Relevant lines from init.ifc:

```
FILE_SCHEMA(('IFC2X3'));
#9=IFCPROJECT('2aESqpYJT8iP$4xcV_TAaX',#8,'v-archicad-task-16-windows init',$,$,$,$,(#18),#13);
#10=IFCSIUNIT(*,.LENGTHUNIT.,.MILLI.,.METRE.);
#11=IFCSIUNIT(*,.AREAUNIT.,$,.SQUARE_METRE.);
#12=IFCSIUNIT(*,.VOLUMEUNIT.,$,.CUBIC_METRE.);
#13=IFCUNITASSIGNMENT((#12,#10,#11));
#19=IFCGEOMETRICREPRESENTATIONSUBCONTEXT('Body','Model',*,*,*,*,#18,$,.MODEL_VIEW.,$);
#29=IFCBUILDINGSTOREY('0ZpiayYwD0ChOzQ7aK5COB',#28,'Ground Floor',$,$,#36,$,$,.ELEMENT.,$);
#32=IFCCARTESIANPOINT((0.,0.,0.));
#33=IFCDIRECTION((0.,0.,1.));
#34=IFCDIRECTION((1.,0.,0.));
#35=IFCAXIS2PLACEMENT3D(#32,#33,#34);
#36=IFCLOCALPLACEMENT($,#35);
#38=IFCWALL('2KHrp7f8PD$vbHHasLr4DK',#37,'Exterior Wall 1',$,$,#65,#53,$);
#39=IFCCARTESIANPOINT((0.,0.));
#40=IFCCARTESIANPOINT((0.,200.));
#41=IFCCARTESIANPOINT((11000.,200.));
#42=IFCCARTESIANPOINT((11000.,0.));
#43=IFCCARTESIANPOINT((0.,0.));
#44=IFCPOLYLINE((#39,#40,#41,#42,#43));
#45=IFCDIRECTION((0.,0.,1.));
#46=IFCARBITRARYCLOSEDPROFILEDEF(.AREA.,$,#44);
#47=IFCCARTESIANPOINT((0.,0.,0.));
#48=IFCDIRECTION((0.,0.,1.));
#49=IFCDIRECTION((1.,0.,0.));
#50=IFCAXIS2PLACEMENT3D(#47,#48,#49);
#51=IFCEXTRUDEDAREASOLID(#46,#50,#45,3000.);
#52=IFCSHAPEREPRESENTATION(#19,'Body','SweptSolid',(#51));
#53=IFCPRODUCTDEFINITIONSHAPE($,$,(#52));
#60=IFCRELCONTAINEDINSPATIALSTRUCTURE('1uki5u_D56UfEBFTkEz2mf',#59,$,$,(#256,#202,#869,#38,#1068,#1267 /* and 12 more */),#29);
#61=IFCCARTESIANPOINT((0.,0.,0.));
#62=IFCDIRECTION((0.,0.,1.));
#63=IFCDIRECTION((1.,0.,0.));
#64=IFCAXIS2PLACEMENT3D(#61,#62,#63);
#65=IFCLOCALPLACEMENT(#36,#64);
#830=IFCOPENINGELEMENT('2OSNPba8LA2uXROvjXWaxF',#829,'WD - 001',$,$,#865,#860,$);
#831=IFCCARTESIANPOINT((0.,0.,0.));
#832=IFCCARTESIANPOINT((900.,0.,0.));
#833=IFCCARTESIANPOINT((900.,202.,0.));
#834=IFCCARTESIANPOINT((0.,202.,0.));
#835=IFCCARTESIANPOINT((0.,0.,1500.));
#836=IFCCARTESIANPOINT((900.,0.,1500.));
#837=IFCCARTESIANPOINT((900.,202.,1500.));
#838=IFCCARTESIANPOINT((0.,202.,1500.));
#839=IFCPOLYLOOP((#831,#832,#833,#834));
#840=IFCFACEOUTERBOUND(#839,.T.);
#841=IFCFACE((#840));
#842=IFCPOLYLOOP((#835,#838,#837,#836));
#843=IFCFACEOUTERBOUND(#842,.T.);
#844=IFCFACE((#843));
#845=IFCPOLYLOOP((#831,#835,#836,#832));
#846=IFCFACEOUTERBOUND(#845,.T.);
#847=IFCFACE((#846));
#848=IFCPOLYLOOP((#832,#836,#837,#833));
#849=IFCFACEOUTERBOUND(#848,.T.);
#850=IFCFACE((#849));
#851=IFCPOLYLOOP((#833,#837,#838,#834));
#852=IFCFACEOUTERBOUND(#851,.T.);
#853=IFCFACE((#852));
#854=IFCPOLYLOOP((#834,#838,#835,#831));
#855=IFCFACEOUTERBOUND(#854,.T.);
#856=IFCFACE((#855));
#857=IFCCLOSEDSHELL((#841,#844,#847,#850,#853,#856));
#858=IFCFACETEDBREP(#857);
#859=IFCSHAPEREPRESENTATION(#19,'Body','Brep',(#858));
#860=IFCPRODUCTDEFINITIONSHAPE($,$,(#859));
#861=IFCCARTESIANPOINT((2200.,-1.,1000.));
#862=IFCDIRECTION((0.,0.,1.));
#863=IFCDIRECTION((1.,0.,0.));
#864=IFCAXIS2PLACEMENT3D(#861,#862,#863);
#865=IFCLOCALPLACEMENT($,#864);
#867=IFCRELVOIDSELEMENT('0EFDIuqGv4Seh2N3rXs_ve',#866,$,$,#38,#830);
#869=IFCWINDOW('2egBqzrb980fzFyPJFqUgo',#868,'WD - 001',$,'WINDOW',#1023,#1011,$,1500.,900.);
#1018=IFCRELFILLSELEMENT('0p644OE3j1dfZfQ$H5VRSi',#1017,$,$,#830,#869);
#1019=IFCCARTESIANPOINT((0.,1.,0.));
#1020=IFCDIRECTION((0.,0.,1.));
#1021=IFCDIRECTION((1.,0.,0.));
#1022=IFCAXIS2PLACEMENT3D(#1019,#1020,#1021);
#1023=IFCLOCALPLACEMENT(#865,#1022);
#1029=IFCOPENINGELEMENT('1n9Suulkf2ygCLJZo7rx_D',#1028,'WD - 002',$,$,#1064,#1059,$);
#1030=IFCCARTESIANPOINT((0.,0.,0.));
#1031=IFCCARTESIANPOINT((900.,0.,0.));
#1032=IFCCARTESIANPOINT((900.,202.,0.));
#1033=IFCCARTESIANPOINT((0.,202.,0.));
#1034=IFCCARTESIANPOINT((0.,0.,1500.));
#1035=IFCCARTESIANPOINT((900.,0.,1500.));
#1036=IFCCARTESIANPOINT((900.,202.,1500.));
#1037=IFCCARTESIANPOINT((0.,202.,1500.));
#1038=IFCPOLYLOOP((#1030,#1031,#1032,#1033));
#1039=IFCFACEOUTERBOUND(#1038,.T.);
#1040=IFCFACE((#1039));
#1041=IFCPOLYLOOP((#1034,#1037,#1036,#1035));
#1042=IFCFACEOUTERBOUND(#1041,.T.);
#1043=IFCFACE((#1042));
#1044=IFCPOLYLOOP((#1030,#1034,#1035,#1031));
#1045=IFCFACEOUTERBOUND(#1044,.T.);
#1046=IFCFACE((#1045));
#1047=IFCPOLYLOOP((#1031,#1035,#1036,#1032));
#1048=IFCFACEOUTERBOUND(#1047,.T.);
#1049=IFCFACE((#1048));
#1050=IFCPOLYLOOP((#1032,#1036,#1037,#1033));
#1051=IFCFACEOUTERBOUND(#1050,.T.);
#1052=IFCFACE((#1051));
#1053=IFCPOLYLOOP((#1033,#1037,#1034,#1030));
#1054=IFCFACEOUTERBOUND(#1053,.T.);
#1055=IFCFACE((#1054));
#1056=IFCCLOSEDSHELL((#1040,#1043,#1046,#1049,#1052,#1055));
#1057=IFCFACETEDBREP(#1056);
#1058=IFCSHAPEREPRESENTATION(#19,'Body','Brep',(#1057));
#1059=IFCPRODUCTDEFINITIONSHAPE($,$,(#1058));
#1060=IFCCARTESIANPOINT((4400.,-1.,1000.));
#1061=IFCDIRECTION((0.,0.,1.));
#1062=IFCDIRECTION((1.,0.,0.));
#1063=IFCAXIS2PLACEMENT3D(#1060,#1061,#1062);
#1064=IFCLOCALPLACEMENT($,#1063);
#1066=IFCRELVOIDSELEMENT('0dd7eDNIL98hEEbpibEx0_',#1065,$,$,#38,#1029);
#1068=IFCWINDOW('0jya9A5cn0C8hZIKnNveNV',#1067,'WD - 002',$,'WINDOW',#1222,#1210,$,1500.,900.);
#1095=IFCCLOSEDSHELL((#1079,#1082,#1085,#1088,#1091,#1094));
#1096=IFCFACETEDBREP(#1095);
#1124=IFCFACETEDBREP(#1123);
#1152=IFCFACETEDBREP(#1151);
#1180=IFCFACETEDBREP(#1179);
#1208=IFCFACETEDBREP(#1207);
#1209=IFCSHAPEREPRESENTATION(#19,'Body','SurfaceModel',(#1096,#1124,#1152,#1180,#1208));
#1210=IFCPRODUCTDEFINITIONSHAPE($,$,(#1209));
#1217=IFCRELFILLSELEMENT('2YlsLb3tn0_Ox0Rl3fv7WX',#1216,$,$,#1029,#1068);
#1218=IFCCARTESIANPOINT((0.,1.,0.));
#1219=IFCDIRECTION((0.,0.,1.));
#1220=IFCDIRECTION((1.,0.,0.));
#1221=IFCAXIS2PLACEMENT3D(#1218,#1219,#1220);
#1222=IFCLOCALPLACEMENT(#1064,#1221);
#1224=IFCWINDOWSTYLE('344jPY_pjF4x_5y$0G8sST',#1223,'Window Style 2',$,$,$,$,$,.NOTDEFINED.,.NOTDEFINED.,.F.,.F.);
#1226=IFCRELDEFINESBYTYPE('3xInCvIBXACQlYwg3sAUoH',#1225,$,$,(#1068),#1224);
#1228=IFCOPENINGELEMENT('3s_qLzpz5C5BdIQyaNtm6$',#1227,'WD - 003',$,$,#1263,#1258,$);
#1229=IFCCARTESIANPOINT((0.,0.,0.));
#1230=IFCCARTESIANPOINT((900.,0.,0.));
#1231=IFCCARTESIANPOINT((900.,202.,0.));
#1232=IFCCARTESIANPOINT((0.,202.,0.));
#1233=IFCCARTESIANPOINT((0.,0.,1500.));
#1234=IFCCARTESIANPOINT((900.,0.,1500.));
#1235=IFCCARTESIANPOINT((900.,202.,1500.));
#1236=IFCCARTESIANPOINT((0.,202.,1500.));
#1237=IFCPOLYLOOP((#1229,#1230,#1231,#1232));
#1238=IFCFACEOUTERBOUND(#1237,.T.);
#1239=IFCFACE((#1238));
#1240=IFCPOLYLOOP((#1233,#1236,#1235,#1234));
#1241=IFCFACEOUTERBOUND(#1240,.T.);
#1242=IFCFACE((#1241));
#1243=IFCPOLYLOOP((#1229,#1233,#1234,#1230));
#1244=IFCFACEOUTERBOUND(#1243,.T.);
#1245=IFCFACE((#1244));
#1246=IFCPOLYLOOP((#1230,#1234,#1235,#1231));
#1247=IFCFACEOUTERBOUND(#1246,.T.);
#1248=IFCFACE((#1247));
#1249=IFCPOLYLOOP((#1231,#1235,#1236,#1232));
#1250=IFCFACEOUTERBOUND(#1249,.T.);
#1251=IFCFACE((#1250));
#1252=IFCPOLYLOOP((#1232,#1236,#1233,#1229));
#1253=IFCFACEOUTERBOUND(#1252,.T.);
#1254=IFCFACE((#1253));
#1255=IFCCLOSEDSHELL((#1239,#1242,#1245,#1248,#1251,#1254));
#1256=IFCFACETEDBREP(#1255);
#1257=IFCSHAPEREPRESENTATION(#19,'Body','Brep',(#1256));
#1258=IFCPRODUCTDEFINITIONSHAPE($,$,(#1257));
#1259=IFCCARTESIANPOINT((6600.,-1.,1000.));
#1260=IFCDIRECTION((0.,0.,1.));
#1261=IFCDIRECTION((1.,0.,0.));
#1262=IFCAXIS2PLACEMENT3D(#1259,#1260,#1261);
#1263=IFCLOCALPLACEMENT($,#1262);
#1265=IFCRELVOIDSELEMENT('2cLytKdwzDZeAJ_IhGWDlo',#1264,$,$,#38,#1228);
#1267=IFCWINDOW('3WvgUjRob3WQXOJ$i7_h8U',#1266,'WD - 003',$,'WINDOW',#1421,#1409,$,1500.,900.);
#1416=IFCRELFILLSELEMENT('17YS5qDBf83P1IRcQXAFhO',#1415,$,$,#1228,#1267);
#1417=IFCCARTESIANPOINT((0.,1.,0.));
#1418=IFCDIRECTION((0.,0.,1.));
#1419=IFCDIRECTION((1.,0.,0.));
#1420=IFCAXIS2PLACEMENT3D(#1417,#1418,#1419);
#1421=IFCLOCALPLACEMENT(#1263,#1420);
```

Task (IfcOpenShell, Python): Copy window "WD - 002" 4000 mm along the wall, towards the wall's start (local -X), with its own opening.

```python
import ifcopenshell
import ifcopenshell.api.feature
import ifcopenshell.api.geometry
import ifcopenshell.api.root
import ifcopenshell.geom
import ifcopenshell.util.element
import ifcopenshell.util.placement
import ifcopenshell.util.shape
import ifcopenshell.util.unit

model = ifcopenshell.open("init.ifc")
unit_scale = ifcopenshell.util.unit.calculate_unit_scale(model)
settings = ifcopenshell.geom.settings()


def volume(element):
    """Net volume in cubic metres, openings subtracted."""
    shape = ifcopenshell.geom.create_shape(settings, element)
    return ifcopenshell.util.shape.get_volume(shape.geometry)


window = model.by_guid("0jya9A5cn0C8hZIKnNveNV")
opening = window.FillsVoids[0].RelatingOpeningElement
wall = opening.VoidsElements[0].RelatingBuildingElement
before = volume(wall)
shift = ifcopenshell.util.placement.get_local_placement(wall.ObjectPlacement)[:3, 0] * -4 / unit_scale

# copy_class copies the void relationship, type, container and properties, but no geometry.
new_opening = ifcopenshell.api.root.copy_class(model, product=opening)
new_opening.Representation = ifcopenshell.util.element.copy_deep(
    model, opening.Representation, exclude=["IfcGeometricRepresentationContext", "IfcRepresentationMap"]
)
new_window = ifcopenshell.api.root.copy_class(model, product=window)
new_window.Representation = ifcopenshell.util.element.copy_deep(
    model, window.Representation, exclude=["IfcGeometricRepresentationContext", "IfcRepresentationMap"]
)
fills = ifcopenshell.api.feature.add_filling(model, opening=new_opening, element=new_window)
fills.OwnerHistory = new_window.OwnerHistory  # required in IFC2X3

for old, new in ((opening, new_opening), (window, new_window)):
    matrix = ifcopenshell.util.placement.get_local_placement(old.ObjectPlacement)
    matrix[:3, 3] += shift
    ifcopenshell.api.geometry.edit_object_placement(model, product=new, matrix=matrix, is_si=False)

after = volume(wall)

print(f"wall volume {before:.3f} -> {after:.3f} m3")

model.write("init_updated.ifc")
```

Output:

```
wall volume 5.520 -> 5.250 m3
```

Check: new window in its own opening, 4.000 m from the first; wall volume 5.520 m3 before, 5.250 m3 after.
